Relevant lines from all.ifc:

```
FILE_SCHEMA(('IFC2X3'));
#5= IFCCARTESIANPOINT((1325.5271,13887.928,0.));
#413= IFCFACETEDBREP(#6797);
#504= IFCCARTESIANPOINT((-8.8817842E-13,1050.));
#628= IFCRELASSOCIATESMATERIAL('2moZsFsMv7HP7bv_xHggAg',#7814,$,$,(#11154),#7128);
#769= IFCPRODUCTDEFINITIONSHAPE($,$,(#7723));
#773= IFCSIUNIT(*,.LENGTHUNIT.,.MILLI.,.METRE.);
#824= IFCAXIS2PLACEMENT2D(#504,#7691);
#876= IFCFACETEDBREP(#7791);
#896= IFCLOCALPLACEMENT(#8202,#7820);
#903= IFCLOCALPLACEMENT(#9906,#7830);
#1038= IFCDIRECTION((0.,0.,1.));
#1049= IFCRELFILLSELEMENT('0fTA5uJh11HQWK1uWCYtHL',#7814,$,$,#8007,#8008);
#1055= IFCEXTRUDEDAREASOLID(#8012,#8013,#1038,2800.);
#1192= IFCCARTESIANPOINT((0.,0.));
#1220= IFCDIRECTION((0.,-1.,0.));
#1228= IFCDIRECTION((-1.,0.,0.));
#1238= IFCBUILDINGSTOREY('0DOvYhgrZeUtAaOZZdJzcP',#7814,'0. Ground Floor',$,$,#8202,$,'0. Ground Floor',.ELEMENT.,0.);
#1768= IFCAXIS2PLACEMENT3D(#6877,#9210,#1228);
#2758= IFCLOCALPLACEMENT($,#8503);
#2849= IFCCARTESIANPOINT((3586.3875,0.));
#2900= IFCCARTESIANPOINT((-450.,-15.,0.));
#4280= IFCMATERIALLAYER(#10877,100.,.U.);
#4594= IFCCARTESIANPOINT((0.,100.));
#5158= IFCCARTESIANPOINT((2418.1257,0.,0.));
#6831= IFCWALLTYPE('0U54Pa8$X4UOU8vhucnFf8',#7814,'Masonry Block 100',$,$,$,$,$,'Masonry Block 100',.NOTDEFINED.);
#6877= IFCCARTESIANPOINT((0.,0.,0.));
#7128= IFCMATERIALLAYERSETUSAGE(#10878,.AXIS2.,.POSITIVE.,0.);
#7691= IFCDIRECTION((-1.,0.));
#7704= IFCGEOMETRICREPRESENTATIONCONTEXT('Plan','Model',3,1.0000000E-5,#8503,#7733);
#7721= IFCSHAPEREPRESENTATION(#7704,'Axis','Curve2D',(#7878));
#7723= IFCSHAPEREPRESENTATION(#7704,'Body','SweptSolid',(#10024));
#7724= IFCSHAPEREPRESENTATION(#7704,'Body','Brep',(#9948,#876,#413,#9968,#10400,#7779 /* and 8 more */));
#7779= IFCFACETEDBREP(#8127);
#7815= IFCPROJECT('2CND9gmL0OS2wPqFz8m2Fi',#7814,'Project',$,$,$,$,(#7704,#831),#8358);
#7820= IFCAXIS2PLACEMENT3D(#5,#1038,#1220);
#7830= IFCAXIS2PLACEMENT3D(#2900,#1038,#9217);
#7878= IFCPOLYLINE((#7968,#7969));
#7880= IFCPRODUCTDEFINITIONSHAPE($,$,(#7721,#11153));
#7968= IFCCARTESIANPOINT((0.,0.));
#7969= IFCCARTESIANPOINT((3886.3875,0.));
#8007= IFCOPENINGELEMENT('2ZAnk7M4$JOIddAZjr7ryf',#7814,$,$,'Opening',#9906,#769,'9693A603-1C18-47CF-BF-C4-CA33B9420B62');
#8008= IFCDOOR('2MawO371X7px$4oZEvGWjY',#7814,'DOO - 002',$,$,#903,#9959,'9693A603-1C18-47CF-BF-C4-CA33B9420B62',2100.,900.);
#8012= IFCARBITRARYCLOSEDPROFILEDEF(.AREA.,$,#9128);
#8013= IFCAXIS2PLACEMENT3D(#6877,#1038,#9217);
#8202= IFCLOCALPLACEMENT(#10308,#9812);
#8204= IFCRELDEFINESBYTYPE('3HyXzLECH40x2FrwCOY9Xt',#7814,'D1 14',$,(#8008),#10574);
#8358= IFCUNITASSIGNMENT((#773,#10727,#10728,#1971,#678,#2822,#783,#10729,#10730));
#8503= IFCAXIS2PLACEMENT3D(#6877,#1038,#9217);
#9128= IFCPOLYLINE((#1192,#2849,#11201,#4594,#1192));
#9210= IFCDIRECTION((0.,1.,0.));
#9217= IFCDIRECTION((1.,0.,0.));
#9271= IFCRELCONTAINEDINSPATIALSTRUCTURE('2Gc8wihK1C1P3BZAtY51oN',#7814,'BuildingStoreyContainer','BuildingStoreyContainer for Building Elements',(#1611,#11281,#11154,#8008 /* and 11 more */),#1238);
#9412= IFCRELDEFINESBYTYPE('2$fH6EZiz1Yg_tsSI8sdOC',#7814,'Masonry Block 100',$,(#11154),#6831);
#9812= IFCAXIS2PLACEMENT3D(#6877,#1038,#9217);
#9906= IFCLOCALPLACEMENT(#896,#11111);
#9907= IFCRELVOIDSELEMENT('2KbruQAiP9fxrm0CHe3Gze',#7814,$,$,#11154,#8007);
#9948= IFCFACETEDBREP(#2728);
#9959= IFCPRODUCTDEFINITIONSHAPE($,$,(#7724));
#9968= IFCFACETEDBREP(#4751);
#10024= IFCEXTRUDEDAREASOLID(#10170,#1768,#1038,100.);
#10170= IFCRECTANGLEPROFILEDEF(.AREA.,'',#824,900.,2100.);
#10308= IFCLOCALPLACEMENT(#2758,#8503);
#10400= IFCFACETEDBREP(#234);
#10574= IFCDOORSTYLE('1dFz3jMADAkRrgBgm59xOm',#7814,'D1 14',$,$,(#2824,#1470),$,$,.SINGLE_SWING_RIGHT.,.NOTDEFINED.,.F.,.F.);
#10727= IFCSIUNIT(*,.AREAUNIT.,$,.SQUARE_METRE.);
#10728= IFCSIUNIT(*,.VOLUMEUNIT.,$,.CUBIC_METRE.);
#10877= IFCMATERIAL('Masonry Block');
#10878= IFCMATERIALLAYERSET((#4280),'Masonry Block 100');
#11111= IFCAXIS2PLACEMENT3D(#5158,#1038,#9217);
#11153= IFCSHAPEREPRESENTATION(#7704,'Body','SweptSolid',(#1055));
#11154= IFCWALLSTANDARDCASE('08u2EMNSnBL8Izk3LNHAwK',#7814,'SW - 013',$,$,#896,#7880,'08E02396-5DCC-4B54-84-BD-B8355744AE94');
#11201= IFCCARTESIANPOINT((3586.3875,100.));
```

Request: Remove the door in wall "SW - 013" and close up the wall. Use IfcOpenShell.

```python
import ifcopenshell
import ifcopenshell.api.feature
import ifcopenshell.api.root
import ifcopenshell.geom
import ifcopenshell.util.shape

model = ifcopenshell.open("all.ifc")
settings = ifcopenshell.geom.settings()


def volume(element):
    """Net volume in cubic metres, openings subtracted."""
    shape = ifcopenshell.geom.create_shape(settings, element)
    return ifcopenshell.util.shape.get_volume(shape.geometry)


door = model.by_id(8008)
opening = door.FillsVoids[0].RelatingOpeningElement
wall = opening.VoidsElements[0].RelatingBuildingElement
before = volume(wall)

ifcopenshell.api.root.remove_product(model, product=door)
ifcopenshell.api.feature.remove_feature(model, feature=opening)

after = volume(wall)

print(f"wall volume {before:.3f} -> {after:.3f} m3")

model.write("all_rev.ifc")
```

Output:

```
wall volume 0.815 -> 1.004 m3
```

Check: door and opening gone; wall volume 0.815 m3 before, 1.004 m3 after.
